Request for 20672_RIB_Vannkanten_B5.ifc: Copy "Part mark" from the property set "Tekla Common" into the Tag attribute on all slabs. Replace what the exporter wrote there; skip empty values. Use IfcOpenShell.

First a look at what the model holds.

```python
import ifcopenshell
import ifcopenshell.util.element

model = ifcopenshell.open("20672_RIB_Vannkanten_B5.ifc")
print(model.schema)
slabs = model.by_type("IfcSlab")
print(len(slabs), "slabs")
for e in slabs[:8]:
    source = ifcopenshell.util.element.get_pset(e, "Tekla Common", "Part mark")
    target = e.Tag
    print(e.id(), repr(source), repr(target), sep=" | ")
```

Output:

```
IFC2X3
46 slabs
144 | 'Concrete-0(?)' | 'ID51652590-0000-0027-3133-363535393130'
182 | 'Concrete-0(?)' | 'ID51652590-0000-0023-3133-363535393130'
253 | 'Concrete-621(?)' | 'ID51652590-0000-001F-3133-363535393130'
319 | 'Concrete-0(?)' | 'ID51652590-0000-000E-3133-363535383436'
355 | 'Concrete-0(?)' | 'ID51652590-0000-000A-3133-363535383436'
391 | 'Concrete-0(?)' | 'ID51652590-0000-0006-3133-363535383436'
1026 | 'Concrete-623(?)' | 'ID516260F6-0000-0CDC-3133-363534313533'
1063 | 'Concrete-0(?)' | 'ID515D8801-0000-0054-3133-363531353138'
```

```python
import ifcopenshell
import ifcopenshell.util.element

model = ifcopenshell.open("20672_RIB_Vannkanten_B5.ifc")

count = 0
for e in model.by_type("IfcSlab"):
    value = ifcopenshell.util.element.get_pset(e, "Tekla Common", "Part mark")
    current = e.Tag
    if not value or not value.strip() or current == value:
        continue
    e.Tag = value
    count += 1

print(count, "slabs updated")

model.write("20672_RIB_Vannkanten_B5_rev.ifc")
```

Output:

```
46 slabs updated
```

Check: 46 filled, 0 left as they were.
